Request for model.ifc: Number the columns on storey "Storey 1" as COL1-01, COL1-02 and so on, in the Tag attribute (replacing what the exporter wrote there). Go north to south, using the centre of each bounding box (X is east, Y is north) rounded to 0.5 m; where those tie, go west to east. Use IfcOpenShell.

First a look at what the model holds.

```python
import ifcopenshell
import ifcopenshell.util.element
import ifcopenshell.util.placement

model = ifcopenshell.open("model.ifc")
print(model.schema)
storey = next(s for s in model.by_type("IfcBuildingStorey") if s.Name == "Storey 1")
columns = [e for e in ifcopenshell.util.element.get_decomposition(storey) if e.is_a("IfcColumn")]
for e in sorted(columns, key=lambda e: e.id()):
    origin = ifcopenshell.util.placement.get_local_placement(e.ObjectPlacement)[:3, 3]
    print(e.id(), e.Tag, e.Name, origin.round(2) + 0.0, sep=" | ")
```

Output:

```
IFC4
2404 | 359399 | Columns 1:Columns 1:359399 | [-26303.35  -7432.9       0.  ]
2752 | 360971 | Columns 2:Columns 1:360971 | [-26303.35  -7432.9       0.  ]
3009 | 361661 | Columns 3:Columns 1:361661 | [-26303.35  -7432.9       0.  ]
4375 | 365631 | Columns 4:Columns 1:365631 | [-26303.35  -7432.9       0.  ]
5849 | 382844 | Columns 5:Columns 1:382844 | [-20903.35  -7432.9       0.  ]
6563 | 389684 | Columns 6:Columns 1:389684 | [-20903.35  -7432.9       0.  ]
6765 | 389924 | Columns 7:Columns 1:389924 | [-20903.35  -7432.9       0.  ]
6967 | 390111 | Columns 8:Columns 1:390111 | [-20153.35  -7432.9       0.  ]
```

```python
import ifcopenshell
import ifcopenshell.geom
import ifcopenshell.util.element
import ifcopenshell.util.shape

model = ifcopenshell.open("model.ifc")
settings = ifcopenshell.geom.settings()
settings.set("use-world-coords", True)


def centre(element):
    shape = ifcopenshell.geom.create_shape(settings, element)
    return ifcopenshell.util.shape.get_bbox_centroid(shape.geometry)


storey = next(s for s in model.by_type("IfcBuildingStorey") if s.Name == "Storey 1")
columns = [e for e in ifcopenshell.util.element.get_decomposition(storey) if e.is_a("IfcColumn")]

# Insertion points can sit at a corner or the storey origin, so sort by the geometry (in metres).
centres = {e: centre(e) for e in columns}
columns.sort(key=lambda e: (-round(centres[e][1] / 0.5), centres[e][0]))

for i, e in enumerate(columns, start=1):
    number = f"COL1-{i:02d}"
    e.Tag = number
    print(e.id(), number)

model.write("model_updated.ifc")
```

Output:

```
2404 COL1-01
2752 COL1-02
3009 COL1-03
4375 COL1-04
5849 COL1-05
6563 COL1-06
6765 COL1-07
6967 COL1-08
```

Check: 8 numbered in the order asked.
